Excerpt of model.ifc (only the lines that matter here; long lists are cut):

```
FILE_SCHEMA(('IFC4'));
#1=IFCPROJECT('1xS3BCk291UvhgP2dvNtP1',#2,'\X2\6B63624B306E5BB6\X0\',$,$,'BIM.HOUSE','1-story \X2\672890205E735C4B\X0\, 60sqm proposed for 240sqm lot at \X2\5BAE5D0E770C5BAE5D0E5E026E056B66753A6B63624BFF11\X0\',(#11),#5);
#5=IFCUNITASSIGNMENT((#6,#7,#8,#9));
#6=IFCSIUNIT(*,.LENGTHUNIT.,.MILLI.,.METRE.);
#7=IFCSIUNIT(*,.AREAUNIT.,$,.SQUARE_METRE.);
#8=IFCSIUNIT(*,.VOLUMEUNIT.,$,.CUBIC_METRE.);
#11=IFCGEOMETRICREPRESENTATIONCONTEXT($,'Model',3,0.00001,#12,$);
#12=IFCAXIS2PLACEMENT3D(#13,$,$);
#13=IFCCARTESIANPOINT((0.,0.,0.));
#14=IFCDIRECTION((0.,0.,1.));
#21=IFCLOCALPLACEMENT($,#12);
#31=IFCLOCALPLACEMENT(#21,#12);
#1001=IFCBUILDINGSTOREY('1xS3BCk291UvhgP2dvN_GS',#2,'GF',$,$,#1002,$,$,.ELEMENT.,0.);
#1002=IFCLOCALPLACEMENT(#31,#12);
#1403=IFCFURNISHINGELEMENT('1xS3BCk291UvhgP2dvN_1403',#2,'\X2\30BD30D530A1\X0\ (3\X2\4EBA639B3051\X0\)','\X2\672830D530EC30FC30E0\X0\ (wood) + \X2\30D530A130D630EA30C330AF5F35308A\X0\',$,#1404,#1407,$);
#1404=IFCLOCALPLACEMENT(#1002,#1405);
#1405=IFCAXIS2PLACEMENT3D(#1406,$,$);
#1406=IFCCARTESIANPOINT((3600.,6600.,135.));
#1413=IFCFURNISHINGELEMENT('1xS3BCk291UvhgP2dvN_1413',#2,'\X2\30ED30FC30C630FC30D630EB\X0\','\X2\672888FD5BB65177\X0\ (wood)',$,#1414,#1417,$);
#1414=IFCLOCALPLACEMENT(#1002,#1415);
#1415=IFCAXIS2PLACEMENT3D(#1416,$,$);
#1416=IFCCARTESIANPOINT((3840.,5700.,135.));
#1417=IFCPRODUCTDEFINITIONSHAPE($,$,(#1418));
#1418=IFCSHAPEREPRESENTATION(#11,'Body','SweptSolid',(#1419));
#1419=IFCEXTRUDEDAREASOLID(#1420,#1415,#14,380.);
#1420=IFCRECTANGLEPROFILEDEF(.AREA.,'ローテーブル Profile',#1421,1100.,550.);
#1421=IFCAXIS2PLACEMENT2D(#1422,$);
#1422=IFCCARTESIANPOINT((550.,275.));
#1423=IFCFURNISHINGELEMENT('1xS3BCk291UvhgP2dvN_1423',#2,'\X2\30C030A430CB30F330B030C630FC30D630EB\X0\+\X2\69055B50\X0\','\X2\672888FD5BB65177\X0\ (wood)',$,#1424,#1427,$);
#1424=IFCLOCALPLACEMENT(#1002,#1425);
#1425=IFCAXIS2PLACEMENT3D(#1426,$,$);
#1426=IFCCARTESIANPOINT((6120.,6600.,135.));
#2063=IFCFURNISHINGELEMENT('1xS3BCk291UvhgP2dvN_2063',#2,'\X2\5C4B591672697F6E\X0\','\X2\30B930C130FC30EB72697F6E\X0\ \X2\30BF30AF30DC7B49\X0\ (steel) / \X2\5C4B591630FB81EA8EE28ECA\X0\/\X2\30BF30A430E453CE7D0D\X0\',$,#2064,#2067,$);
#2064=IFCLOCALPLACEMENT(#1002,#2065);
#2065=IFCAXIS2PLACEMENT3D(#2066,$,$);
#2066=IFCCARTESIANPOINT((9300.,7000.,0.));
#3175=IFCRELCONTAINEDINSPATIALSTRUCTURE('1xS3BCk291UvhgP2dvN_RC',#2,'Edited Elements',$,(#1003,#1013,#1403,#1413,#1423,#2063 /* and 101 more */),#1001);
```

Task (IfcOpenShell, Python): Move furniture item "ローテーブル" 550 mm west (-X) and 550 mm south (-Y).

```python
import ifcopenshell
import ifcopenshell.api.geometry
import ifcopenshell.util.placement
import ifcopenshell.util.unit

model = ifcopenshell.open("model.ifc")
unit_scale = ifcopenshell.util.unit.calculate_unit_scale(model)

item = model.by_id(1413)
matrix = ifcopenshell.util.placement.get_local_placement(item.ObjectPlacement)
matrix[0, 3] -= 0.55 / unit_scale
matrix[1, 3] -= 0.55 / unit_scale
ifcopenshell.api.geometry.edit_object_placement(model, product=item, matrix=matrix, is_si=False)

print(ifcopenshell.util.placement.get_local_placement(item.ObjectPlacement).round(3) + 0.0)

model.write("model_updated.ifc")
```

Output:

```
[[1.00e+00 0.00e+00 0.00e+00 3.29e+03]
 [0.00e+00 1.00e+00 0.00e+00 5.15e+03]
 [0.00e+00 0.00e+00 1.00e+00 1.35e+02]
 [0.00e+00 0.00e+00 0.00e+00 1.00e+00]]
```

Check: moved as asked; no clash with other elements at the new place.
